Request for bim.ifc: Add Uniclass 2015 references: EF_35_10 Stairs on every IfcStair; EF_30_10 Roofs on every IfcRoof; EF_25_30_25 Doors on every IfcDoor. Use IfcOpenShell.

First a look at what the model holds.

```python
import ifcopenshell

model = ifcopenshell.open("bim.ifc")
print(model.schema)
print("classifications:", [c.Name for c in model.by_type("IfcClassification")])
for ifc_class in ("IfcDoor", "IfcRoof", "IfcStair", "IfcWall", "IfcWindow"):
    print(ifc_class, len(model.by_type(ifc_class)))
```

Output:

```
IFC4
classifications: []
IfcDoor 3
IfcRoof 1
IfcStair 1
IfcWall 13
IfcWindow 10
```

```python
import ifcopenshell
import ifcopenshell.api.classification

model = ifcopenshell.open("bim.ifc")

system = ifcopenshell.api.classification.add_classification(model, classification="Uniclass 2015")

codes = {
    "IfcStair": ("EF_35_10", "Stairs"),
    "IfcRoof": ("EF_30_10", "Roofs"),
    "IfcDoor": ("EF_25_30_25", "Doors"),
}
for ifc_class, (code, name) in codes.items():
    products = model.by_type(ifc_class)
    ifcopenshell.api.classification.add_reference(
        model, products=products, classification=system, identification=code, name=name
    )
    print(code, len(products))

model.write("bim_rev.ifc")
```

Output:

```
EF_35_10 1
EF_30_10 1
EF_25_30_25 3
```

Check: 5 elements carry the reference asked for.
